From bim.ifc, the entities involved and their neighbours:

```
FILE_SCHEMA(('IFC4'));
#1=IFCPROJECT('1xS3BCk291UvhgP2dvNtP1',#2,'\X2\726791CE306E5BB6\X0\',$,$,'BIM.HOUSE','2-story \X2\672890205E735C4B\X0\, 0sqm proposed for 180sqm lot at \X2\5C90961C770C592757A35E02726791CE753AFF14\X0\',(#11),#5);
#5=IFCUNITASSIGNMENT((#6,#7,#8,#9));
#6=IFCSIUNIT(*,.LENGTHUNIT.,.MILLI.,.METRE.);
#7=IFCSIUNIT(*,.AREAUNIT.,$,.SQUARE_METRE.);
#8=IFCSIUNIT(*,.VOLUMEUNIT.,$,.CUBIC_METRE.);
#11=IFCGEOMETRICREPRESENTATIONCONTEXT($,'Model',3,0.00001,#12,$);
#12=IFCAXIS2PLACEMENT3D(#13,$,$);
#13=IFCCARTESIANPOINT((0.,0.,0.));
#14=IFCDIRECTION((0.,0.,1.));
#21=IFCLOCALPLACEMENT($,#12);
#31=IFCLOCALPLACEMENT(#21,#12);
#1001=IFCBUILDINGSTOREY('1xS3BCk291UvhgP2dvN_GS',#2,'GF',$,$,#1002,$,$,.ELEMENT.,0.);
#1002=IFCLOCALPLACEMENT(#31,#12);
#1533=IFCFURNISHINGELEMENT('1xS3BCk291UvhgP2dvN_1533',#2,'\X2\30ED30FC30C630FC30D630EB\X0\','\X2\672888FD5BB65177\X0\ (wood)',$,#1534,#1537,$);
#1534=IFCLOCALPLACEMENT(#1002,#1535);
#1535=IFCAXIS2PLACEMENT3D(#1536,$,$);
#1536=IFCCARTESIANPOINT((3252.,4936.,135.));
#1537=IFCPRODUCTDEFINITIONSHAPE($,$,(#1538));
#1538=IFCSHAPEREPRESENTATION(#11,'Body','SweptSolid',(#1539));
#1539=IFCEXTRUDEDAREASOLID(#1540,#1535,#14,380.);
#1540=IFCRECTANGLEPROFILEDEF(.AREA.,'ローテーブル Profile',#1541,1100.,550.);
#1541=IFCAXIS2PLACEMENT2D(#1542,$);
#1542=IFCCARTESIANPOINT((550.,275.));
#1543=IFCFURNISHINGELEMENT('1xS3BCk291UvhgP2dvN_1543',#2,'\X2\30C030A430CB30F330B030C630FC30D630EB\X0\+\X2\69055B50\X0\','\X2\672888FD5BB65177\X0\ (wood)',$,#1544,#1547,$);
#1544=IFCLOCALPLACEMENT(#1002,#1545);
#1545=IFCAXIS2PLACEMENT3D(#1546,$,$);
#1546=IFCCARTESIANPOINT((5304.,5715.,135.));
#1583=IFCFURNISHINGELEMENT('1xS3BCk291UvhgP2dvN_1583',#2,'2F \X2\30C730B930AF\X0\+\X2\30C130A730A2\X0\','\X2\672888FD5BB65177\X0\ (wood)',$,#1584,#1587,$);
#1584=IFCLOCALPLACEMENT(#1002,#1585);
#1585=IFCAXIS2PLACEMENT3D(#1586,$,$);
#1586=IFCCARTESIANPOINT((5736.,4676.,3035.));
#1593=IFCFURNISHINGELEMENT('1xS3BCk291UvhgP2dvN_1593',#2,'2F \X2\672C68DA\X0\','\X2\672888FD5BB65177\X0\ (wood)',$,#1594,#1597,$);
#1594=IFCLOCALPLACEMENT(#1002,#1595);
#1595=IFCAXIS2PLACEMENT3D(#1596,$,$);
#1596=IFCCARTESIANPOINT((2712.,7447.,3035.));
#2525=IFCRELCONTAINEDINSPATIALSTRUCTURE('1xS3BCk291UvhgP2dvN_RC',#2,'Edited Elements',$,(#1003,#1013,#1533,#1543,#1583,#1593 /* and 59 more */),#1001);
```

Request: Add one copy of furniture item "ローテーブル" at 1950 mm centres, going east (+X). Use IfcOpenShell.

```python
import numpy as np
import ifcopenshell
import ifcopenshell.api.geometry
import ifcopenshell.api.root
import ifcopenshell.util.element
import ifcopenshell.util.placement
import ifcopenshell.util.unit

model = ifcopenshell.open("bim.ifc")
unit_scale = ifcopenshell.util.unit.calculate_unit_scale(model)


def reuse_history(source, copy):
    """copy_class also copies each property set's owner history, people and application; keep the originals."""
    for rel in copy.IsDefinedBy:
        if rel.is_a("IfcRelDefinesByProperties") and (history := rel.RelatingPropertyDefinition.OwnerHistory):
            rel.RelatingPropertyDefinition.OwnerHistory = source.OwnerHistory
            ifcopenshell.util.element.remove_deep2(model, history)


source = model.by_id(1533)
base = ifcopenshell.util.placement.get_local_placement(source.ObjectPlacement)
step = np.array([1.0, 0.0, 0.0]) * 1.95 / unit_scale

for i in range(1, 2):
    copy = ifcopenshell.api.root.copy_class(model, product=source)
    copy.Representation = ifcopenshell.util.element.copy_deep(
        model, source.Representation, exclude=["IfcGeometricRepresentationContext", "IfcRepresentationMap"]
    )
    reuse_history(source, copy)
    matrix = base.copy()
    matrix[:3, 3] += i * step
    print("added at", matrix[:3, 3].round(3) + 0.0)
    ifcopenshell.api.geometry.edit_object_placement(model, product=copy, matrix=matrix, is_si=False)

model.write("bim_v2.ifc")
```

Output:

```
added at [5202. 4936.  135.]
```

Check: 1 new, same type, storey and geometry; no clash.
